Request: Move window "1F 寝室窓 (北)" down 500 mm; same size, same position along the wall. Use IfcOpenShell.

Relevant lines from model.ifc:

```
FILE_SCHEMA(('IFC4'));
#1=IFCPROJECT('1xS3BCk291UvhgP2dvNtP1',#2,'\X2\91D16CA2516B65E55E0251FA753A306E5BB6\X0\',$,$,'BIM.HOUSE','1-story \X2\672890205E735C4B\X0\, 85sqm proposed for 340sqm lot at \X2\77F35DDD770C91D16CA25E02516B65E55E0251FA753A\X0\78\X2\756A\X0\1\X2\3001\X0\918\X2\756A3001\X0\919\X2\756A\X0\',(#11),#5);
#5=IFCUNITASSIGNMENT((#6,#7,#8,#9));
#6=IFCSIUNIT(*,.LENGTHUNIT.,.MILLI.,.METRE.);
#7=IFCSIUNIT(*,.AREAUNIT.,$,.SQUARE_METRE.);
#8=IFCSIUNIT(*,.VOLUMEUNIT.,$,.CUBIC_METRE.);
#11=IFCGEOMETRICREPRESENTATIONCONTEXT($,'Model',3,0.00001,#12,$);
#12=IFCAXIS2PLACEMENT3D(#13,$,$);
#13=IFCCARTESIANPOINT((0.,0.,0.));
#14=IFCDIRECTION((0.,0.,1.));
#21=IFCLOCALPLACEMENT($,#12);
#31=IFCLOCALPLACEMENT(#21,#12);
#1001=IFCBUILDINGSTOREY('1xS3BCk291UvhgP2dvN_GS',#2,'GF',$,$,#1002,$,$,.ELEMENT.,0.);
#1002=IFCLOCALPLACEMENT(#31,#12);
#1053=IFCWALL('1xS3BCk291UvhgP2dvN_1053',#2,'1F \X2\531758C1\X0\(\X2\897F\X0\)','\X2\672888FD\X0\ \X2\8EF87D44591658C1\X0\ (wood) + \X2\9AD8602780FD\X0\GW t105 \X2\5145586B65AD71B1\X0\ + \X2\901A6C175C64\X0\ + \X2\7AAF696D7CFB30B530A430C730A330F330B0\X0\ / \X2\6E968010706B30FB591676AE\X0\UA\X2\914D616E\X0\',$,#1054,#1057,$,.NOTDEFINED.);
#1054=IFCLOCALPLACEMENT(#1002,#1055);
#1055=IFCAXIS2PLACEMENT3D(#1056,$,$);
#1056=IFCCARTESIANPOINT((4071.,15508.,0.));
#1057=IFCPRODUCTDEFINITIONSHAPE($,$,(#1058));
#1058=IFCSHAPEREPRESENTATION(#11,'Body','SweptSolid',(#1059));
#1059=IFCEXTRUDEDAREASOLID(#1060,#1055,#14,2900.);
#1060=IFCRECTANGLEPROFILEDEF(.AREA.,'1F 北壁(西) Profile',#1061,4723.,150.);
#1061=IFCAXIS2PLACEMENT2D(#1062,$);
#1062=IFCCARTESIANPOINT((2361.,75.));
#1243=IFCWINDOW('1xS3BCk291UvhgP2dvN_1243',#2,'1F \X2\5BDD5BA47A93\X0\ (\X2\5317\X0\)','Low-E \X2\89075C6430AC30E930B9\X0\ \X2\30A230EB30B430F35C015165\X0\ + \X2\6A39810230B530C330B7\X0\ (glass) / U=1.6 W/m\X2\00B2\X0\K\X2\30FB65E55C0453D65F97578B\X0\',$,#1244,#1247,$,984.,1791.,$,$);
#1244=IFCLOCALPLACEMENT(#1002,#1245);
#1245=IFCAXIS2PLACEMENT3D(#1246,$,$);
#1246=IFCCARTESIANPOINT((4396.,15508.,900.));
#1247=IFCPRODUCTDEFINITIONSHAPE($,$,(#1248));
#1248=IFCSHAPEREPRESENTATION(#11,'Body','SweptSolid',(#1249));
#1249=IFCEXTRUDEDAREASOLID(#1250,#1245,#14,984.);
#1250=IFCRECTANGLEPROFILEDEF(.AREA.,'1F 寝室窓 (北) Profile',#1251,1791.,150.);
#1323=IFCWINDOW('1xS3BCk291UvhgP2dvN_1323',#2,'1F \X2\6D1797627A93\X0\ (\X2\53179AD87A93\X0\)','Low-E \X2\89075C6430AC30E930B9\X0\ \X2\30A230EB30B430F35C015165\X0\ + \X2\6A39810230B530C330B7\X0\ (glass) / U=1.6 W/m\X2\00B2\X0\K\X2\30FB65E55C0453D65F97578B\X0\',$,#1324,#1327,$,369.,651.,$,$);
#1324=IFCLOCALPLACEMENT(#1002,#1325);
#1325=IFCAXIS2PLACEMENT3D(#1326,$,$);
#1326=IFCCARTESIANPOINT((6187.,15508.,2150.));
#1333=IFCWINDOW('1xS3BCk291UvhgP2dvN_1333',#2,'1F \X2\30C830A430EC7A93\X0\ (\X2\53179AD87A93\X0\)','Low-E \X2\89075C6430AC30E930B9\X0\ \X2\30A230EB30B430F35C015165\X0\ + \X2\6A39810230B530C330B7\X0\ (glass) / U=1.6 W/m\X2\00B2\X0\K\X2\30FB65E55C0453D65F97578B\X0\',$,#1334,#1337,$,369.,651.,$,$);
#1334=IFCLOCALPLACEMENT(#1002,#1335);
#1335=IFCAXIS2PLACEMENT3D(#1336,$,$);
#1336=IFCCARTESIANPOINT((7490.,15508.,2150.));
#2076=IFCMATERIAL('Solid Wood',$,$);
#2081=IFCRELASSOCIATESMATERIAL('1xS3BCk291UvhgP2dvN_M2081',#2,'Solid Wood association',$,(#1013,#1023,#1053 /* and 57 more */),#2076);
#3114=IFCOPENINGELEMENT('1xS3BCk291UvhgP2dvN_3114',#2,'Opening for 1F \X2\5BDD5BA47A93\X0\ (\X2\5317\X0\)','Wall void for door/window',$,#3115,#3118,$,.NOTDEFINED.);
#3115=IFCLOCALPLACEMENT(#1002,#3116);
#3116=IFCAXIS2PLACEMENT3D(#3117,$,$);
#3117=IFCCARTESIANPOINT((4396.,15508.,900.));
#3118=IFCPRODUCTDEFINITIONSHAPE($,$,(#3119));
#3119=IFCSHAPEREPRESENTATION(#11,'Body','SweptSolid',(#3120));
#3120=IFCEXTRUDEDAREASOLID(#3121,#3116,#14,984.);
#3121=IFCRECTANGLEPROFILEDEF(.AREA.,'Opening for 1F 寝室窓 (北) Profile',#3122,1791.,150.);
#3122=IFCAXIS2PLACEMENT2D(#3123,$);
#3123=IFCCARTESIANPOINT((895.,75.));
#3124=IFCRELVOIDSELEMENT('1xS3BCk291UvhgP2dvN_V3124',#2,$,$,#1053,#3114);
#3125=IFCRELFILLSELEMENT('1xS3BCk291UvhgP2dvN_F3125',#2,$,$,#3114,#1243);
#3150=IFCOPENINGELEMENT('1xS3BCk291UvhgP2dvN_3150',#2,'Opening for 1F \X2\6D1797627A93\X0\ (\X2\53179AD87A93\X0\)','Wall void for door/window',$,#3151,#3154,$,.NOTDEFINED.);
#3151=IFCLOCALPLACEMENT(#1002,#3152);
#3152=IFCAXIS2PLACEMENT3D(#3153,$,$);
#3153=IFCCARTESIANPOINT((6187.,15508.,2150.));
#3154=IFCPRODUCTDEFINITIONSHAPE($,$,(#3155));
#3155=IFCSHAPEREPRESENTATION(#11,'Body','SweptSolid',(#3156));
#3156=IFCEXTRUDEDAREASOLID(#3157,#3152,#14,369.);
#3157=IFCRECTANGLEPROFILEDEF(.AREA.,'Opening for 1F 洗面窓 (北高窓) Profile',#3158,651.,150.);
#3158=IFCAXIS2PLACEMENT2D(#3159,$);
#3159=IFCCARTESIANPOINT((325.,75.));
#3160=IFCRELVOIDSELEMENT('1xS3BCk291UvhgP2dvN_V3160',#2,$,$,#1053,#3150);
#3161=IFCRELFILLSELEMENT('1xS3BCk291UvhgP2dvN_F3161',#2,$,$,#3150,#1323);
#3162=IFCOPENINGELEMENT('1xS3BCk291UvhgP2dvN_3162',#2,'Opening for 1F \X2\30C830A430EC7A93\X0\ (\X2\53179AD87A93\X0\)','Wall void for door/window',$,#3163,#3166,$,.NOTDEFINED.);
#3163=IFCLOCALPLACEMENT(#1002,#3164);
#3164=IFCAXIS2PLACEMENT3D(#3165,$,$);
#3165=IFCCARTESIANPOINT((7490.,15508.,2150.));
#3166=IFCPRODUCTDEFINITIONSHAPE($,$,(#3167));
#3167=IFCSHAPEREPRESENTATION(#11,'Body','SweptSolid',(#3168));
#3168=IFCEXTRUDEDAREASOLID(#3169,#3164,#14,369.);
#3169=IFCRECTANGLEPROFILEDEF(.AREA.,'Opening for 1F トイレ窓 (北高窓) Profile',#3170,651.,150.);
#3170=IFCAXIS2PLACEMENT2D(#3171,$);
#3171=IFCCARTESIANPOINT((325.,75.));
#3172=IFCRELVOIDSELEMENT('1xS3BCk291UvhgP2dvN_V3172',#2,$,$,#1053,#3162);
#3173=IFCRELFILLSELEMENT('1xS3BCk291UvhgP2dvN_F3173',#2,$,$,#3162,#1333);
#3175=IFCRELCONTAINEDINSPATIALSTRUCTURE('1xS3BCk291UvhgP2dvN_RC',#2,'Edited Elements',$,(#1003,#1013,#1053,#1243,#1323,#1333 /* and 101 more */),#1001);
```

```python
import numpy as np
import ifcopenshell
import ifcopenshell.api.geometry
import ifcopenshell.util.placement
import ifcopenshell.util.unit

model = ifcopenshell.open("model.ifc")
unit_scale = ifcopenshell.util.unit.calculate_unit_scale(model)

window = model.by_guid("1xS3BCk291UvhgP2dvN_1243")
opening = window.FillsVoids[0].RelatingOpeningElement
dz = -500.0

shift = np.array([0.0, 0.0, dz])
# The window is not placed relative to its opening, so move both.
for product in (opening, window):
    matrix = ifcopenshell.util.placement.get_local_placement(product.ObjectPlacement)
    matrix[:3, 3] += shift
    ifcopenshell.api.geometry.edit_object_placement(model, product=product, matrix=matrix, is_si=False)

print(f"moved by {dz * unit_scale:+.3f} m")

model.write("model_v2.ifc")
```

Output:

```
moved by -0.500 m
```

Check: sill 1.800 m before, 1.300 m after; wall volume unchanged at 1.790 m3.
